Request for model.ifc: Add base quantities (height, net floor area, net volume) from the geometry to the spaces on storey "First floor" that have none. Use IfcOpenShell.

First a look at what the model holds.

```python
import ifcopenshell
import ifcopenshell.util.element
import ifcopenshell.util.unit

model = ifcopenshell.open("model.ifc")
print(model.schema)
for unit_type in ("LENGTHUNIT", "AREAUNIT", "VOLUMEUNIT"):
    print(unit_type, ifcopenshell.util.unit.calculate_unit_scale(model, unit_type))
storey = next(s for s in model.by_type("IfcBuildingStorey") if s.Name == "First floor")
spaces = [e for e in ifcopenshell.util.element.get_decomposition(storey) if e.is_a("IfcSpace")]
for e in sorted(spaces, key=lambda e: e.id()):
    print(e.id(), e.is_a(), e.Name, list(ifcopenshell.util.element.get_psets(e, qtos_only=True)), sep=" | ")
```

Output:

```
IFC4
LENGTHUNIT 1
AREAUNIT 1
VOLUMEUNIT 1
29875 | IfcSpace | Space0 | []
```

```python
import ifcopenshell
import ifcopenshell.api.pset
import ifcopenshell.geom
import ifcopenshell.util.element
import ifcopenshell.util.shape
import ifcopenshell.util.unit

model = ifcopenshell.open("model.ifc")
unit_scale = ifcopenshell.util.unit.calculate_unit_scale(model)
area_scale = ifcopenshell.util.unit.calculate_unit_scale(model, "AREAUNIT")
volume_scale = ifcopenshell.util.unit.calculate_unit_scale(model, "VOLUMEUNIT")
settings = ifcopenshell.geom.settings()

storey = next(s for s in model.by_type("IfcBuildingStorey") if s.Name == "First floor")
spaces = [e for e in ifcopenshell.util.element.get_decomposition(storey) if e.is_a("IfcSpace")]

for e in sorted(spaces, key=lambda e: e.id()):
    if ifcopenshell.util.element.get_psets(e, qtos_only=True, should_inherit=False):
        continue
    # Geometry comes back in metres, in the element's own axes.
    shape = ifcopenshell.geom.create_shape(settings, e)
    values = {
        "Height": ifcopenshell.util.shape.get_z(shape.geometry) / unit_scale,
        "NetFloorArea": ifcopenshell.util.shape.get_footprint_area(shape.geometry) / area_scale,
        "NetVolume": ifcopenshell.util.shape.get_volume(shape.geometry) / volume_scale,
    }
    qto = ifcopenshell.api.pset.add_qto(model, product=e, name="Qto_SpaceBaseQuantities")
    ifcopenshell.api.pset.edit_qto(model, qto=qto, properties=values)
    print(e.id(), {k: round(v, 3) for k, v in values.items()})

model.write("model_rev.ifc")
```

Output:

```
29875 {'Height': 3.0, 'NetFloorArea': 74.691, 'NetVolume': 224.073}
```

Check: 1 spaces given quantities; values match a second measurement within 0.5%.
